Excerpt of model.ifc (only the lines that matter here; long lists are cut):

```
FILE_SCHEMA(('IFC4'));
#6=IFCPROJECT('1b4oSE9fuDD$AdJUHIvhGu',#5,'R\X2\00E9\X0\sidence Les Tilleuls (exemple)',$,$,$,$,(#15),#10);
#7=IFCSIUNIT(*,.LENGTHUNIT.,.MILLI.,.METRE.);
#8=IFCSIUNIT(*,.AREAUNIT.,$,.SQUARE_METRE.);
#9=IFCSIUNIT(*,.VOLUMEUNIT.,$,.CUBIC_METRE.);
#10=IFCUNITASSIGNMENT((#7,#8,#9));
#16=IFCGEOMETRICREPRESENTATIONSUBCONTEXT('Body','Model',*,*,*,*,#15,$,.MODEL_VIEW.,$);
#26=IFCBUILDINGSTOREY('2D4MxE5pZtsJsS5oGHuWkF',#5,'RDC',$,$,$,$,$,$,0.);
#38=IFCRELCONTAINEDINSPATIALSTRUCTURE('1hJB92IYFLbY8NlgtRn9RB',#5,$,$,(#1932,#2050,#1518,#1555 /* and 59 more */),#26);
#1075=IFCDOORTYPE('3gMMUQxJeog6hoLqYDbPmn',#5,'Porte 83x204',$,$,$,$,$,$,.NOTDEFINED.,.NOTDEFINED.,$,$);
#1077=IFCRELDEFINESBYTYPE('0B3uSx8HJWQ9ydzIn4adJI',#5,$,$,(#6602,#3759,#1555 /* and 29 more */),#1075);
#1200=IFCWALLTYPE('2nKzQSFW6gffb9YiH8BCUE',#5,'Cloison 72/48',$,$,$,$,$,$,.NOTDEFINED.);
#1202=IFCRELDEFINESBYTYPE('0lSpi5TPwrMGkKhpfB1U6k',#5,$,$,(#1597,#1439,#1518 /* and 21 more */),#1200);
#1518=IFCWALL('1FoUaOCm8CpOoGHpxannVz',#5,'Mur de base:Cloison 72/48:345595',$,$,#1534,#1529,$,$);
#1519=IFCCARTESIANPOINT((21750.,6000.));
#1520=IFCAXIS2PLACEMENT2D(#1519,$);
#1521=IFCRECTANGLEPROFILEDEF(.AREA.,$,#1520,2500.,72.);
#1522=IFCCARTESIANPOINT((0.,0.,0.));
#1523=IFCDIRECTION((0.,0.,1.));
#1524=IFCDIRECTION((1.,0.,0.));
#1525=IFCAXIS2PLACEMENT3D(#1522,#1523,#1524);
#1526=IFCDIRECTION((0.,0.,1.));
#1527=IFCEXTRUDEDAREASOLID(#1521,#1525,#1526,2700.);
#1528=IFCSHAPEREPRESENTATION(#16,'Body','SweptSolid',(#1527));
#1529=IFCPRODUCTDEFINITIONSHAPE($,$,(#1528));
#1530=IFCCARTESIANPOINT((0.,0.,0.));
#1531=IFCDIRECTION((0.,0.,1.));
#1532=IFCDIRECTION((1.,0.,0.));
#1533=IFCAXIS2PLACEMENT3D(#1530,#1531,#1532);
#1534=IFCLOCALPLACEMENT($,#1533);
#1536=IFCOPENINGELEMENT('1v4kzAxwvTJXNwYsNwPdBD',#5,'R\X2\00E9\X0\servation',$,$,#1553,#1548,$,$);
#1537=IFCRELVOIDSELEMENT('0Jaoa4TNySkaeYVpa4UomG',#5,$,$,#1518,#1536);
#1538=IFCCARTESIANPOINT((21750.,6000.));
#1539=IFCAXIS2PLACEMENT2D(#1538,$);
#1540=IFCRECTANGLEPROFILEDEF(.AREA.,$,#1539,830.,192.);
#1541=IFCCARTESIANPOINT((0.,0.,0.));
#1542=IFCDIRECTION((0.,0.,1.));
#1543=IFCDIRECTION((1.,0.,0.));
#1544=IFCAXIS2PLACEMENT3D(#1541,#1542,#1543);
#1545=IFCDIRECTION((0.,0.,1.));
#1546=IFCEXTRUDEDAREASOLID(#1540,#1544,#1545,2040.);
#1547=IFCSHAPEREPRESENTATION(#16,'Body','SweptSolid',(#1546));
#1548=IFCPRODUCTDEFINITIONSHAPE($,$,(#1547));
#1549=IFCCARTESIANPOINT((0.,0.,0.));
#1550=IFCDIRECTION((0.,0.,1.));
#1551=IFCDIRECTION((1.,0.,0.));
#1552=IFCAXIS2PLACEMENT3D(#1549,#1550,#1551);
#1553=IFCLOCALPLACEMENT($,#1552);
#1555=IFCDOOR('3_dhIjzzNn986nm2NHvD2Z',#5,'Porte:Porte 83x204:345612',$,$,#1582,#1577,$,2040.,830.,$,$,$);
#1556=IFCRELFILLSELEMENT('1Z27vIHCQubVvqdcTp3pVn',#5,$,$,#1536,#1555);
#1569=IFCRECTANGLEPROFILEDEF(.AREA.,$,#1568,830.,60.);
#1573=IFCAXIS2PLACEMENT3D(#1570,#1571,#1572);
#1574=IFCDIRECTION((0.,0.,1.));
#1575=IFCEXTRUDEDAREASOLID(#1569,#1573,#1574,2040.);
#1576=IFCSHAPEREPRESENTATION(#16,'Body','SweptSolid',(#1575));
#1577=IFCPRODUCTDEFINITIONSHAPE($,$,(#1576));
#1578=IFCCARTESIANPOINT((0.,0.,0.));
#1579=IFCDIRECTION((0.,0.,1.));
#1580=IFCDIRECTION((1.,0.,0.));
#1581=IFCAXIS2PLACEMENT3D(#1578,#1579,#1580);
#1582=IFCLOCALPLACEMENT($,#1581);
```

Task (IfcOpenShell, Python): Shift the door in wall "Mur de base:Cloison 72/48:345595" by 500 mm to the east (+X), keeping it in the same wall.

```python
import ifcopenshell
import ifcopenshell.api.geometry
import ifcopenshell.util.placement
import ifcopenshell.util.unit

model = ifcopenshell.open("model.ifc")
unit_scale = ifcopenshell.util.unit.calculate_unit_scale(model)

door = model.by_guid("3_dhIjzzNn986nm2NHvD2Z")
opening = door.FillsVoids[0].RelatingOpeningElement
wall = opening.VoidsElements[0].RelatingBuildingElement

wall_matrix = ifcopenshell.util.placement.get_local_placement(wall.ObjectPlacement)
shift = wall_matrix[:3, 0] * 0.5 / unit_scale
before = ifcopenshell.util.placement.get_local_placement(door.ObjectPlacement)[:3, 3].copy()

# The door is not placed relative to its opening, so move both.
for product in (opening, door):
    matrix = ifcopenshell.util.placement.get_local_placement(product.ObjectPlacement)
    matrix[:3, 3] += shift
    ifcopenshell.api.geometry.edit_object_placement(model, product=product, matrix=matrix, is_si=False)

after = ifcopenshell.util.placement.get_local_placement(door.ObjectPlacement)[:3, 3]
print("door moved by", (after - before).round(3) + 0.0)

model.write("model-out.ifc")
```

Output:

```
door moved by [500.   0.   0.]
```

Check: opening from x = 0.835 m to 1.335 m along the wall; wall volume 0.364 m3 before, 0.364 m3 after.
